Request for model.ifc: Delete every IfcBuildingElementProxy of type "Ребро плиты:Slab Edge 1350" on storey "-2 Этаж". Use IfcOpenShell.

First a look at what the model holds.

```python
import ifcopenshell
import ifcopenshell.util.element

model = ifcopenshell.open("model.ifc")
print(model.schema)
storey = next(s for s in model.by_type("IfcBuildingStorey") if s.Name == "-2 Этаж")
proxies = [e for e in ifcopenshell.util.element.get_decomposition(storey) if e.is_a("IfcBuildingElementProxy")]
seen = {}
for e in proxies:
    element_type = ifcopenshell.util.element.get_type(e)
    name = element_type.Name if element_type not in (None, e) else None
    seen[name] = seen.get(name, 0) + 1
for name, count in sorted(seen.items(), key=str):
    print(count, "x", name)
```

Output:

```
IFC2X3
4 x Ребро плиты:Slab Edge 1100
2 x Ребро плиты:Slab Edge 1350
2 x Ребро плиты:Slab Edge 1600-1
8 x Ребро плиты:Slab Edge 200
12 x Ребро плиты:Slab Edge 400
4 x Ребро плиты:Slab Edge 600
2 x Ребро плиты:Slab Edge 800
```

```python
import ifcopenshell
import ifcopenshell.api.root
import ifcopenshell.util.element

model = ifcopenshell.open("model.ifc")

storey = next(s for s in model.by_type("IfcBuildingStorey") if s.Name == "-2 Этаж")
proxies = [e for e in ifcopenshell.util.element.get_decomposition(storey) if e.is_a("IfcBuildingElementProxy")]
targets = [e for e in proxies if (t := ifcopenshell.util.element.get_type(e)) not in (None, e) and t.Name == "Ребро плиты:Slab Edge 1350"]

for e in targets:
    ifcopenshell.api.root.remove_product(model, product=e)
print(len(targets), "removed")

model.write("model-out.ifc")
```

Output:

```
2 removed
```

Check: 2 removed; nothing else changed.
